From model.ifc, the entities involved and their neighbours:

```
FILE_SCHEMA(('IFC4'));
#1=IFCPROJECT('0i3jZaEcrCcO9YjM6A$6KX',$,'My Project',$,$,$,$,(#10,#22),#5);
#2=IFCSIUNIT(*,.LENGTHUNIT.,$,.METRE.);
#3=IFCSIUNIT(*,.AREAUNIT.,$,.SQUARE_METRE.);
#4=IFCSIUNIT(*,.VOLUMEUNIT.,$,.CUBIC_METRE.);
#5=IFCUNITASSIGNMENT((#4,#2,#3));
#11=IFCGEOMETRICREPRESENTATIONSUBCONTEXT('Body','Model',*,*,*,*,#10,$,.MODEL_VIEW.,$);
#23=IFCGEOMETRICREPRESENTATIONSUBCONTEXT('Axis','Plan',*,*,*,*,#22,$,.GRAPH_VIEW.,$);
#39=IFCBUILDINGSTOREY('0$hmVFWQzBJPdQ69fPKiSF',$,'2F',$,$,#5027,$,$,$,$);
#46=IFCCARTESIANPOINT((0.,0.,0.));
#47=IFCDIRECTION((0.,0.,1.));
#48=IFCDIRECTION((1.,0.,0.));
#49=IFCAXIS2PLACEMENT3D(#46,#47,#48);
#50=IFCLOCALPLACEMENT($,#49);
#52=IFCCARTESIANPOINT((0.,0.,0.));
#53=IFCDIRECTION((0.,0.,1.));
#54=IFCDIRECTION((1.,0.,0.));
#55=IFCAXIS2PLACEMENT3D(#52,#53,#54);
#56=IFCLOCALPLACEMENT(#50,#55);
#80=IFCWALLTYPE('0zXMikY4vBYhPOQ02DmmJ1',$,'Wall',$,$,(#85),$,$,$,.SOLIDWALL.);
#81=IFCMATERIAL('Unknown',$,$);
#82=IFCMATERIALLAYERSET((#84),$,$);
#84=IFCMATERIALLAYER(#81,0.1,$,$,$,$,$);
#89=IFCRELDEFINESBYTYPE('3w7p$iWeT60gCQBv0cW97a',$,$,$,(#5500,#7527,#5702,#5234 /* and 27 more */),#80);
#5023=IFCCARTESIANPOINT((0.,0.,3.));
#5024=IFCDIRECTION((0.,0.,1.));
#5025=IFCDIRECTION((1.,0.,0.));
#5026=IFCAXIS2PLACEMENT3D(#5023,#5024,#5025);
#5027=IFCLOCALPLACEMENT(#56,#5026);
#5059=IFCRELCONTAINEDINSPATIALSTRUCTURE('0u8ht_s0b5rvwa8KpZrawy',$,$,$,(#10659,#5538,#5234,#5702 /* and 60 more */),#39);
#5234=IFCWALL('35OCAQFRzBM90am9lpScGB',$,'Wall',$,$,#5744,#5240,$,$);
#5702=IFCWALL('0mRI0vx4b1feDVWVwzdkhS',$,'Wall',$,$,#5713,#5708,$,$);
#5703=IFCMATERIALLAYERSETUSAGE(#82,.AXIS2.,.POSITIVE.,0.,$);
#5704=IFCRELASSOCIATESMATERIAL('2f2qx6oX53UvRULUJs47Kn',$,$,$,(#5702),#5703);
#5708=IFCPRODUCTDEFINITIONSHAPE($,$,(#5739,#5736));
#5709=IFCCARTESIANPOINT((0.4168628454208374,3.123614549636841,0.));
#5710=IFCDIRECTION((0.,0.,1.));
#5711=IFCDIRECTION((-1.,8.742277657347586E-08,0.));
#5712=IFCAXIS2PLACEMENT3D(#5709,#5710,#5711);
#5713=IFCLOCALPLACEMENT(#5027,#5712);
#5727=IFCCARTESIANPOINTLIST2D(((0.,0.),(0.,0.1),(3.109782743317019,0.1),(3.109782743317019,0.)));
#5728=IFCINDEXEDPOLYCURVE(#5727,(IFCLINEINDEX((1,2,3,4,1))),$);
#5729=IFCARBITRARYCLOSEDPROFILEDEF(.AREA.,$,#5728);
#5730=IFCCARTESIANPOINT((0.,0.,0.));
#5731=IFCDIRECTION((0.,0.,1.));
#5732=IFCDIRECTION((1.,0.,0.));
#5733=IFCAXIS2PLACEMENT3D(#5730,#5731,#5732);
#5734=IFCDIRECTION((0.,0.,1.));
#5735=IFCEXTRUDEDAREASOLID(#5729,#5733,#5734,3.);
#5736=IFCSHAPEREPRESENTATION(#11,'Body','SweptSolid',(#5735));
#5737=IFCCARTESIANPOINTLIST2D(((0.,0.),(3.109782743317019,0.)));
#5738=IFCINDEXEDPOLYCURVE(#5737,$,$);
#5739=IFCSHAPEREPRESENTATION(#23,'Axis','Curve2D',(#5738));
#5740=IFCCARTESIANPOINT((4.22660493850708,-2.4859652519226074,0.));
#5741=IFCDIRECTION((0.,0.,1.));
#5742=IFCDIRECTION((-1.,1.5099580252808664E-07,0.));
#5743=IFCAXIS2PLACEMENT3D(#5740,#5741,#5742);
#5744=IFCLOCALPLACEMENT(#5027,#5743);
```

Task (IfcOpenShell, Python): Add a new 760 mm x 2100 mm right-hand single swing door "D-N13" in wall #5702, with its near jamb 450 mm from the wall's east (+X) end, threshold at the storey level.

```python
import numpy as np
import ifcopenshell
import ifcopenshell.api.feature
import ifcopenshell.api.geometry
import ifcopenshell.api.root
import ifcopenshell.api.spatial
import ifcopenshell.geom
import ifcopenshell.util.element
import ifcopenshell.util.placement
import ifcopenshell.util.representation
import ifcopenshell.util.shape
import ifcopenshell.util.unit

model = ifcopenshell.open("model.ifc")
unit_scale = ifcopenshell.util.unit.calculate_unit_scale(model)
settings = ifcopenshell.geom.settings()


def volume(element):
    """Net volume in cubic metres, openings subtracted."""
    shape = ifcopenshell.geom.create_shape(settings, element)
    return ifcopenshell.util.shape.get_volume(shape.geometry)


wall = model.by_guid("0mRI0vx4b1feDVWVwzdkhS")
storey = ifcopenshell.util.element.get_container(wall, ifc_class="IfcBuildingStorey")
context = ifcopenshell.util.representation.get_context(model, "Model", "Body", "MODEL_VIEW")
before = volume(wall)

width, height, from_end, sill = 0.76, 2.1, 0.45, 0.0  # metres

# The wall runs along its own X axis, and the end named is its -X end.
wall_shape = ifcopenshell.geom.create_shape(settings, wall)
x, y, z = ifcopenshell.util.shape.get_vertices(wall_shape.geometry).T
start = x.min() + from_end
face, thickness = float(y.min()), float(y.max() - y.min())
wall_matrix = ifcopenshell.util.placement.get_local_placement(wall.ObjectPlacement)
level = ifcopenshell.util.placement.get_local_placement(storey.ObjectPlacement)[2, 3]


def in_wall(x, y):
    """Placement at x, y metres in the wall's axes, at sill height."""
    matrix = wall_matrix.copy()
    matrix[:, 3] = wall_matrix @ np.array([x / unit_scale, y / unit_scale, 0.0, 1.0])
    matrix[2, 3] = level + sill / unit_scale
    return matrix


# Opening: a box that overshoots both wall faces by 50 mm.
opening = ifcopenshell.api.root.create_entity(model, ifc_class="IfcOpeningElement", predefined_type="OPENING")
box = ifcopenshell.api.geometry.add_wall_representation(
    model, context=context, length=width, height=height, thickness=thickness + 0.1
)
ifcopenshell.api.geometry.assign_representation(model, product=opening, representation=box)
ifcopenshell.api.geometry.edit_object_placement(model, product=opening, matrix=in_wall(start, face - 0.05), is_si=False)
ifcopenshell.api.feature.add_feature(model, feature=opening, element=wall)

door = ifcopenshell.api.root.create_entity(model, ifc_class="IfcDoor", name="D-N13", predefined_type="DOOR")
door.OverallWidth, door.OverallHeight = width / unit_scale, height / unit_scale
door.OperationType = "SINGLE_SWING_RIGHT"
body = ifcopenshell.api.geometry.add_door_representation(
    model,
    context=context,
    overall_width=door.OverallWidth,
    overall_height=door.OverallHeight,
    operation_type="SINGLE_SWING_RIGHT",
    lining_properties={"LiningDepth": thickness / unit_scale, "ThresholdDepth": thickness / unit_scale},
)
ifcopenshell.api.geometry.assign_representation(model, product=door, representation=body)
ifcopenshell.api.spatial.assign_container(model, products=[door], relating_structure=storey)
ifcopenshell.api.feature.add_filling(model, opening=opening, element=door)

# The lining spans the wall, so the door starts at the wall face.
ifcopenshell.api.geometry.edit_object_placement(model, product=door, matrix=in_wall(start, face), is_si=False)

after = volume(wall)

print(f"wall volume {before:.3f} -> {after:.3f} m3")

model.write("model-out.ifc")
```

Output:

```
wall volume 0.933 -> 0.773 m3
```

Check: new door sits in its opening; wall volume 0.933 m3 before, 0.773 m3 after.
